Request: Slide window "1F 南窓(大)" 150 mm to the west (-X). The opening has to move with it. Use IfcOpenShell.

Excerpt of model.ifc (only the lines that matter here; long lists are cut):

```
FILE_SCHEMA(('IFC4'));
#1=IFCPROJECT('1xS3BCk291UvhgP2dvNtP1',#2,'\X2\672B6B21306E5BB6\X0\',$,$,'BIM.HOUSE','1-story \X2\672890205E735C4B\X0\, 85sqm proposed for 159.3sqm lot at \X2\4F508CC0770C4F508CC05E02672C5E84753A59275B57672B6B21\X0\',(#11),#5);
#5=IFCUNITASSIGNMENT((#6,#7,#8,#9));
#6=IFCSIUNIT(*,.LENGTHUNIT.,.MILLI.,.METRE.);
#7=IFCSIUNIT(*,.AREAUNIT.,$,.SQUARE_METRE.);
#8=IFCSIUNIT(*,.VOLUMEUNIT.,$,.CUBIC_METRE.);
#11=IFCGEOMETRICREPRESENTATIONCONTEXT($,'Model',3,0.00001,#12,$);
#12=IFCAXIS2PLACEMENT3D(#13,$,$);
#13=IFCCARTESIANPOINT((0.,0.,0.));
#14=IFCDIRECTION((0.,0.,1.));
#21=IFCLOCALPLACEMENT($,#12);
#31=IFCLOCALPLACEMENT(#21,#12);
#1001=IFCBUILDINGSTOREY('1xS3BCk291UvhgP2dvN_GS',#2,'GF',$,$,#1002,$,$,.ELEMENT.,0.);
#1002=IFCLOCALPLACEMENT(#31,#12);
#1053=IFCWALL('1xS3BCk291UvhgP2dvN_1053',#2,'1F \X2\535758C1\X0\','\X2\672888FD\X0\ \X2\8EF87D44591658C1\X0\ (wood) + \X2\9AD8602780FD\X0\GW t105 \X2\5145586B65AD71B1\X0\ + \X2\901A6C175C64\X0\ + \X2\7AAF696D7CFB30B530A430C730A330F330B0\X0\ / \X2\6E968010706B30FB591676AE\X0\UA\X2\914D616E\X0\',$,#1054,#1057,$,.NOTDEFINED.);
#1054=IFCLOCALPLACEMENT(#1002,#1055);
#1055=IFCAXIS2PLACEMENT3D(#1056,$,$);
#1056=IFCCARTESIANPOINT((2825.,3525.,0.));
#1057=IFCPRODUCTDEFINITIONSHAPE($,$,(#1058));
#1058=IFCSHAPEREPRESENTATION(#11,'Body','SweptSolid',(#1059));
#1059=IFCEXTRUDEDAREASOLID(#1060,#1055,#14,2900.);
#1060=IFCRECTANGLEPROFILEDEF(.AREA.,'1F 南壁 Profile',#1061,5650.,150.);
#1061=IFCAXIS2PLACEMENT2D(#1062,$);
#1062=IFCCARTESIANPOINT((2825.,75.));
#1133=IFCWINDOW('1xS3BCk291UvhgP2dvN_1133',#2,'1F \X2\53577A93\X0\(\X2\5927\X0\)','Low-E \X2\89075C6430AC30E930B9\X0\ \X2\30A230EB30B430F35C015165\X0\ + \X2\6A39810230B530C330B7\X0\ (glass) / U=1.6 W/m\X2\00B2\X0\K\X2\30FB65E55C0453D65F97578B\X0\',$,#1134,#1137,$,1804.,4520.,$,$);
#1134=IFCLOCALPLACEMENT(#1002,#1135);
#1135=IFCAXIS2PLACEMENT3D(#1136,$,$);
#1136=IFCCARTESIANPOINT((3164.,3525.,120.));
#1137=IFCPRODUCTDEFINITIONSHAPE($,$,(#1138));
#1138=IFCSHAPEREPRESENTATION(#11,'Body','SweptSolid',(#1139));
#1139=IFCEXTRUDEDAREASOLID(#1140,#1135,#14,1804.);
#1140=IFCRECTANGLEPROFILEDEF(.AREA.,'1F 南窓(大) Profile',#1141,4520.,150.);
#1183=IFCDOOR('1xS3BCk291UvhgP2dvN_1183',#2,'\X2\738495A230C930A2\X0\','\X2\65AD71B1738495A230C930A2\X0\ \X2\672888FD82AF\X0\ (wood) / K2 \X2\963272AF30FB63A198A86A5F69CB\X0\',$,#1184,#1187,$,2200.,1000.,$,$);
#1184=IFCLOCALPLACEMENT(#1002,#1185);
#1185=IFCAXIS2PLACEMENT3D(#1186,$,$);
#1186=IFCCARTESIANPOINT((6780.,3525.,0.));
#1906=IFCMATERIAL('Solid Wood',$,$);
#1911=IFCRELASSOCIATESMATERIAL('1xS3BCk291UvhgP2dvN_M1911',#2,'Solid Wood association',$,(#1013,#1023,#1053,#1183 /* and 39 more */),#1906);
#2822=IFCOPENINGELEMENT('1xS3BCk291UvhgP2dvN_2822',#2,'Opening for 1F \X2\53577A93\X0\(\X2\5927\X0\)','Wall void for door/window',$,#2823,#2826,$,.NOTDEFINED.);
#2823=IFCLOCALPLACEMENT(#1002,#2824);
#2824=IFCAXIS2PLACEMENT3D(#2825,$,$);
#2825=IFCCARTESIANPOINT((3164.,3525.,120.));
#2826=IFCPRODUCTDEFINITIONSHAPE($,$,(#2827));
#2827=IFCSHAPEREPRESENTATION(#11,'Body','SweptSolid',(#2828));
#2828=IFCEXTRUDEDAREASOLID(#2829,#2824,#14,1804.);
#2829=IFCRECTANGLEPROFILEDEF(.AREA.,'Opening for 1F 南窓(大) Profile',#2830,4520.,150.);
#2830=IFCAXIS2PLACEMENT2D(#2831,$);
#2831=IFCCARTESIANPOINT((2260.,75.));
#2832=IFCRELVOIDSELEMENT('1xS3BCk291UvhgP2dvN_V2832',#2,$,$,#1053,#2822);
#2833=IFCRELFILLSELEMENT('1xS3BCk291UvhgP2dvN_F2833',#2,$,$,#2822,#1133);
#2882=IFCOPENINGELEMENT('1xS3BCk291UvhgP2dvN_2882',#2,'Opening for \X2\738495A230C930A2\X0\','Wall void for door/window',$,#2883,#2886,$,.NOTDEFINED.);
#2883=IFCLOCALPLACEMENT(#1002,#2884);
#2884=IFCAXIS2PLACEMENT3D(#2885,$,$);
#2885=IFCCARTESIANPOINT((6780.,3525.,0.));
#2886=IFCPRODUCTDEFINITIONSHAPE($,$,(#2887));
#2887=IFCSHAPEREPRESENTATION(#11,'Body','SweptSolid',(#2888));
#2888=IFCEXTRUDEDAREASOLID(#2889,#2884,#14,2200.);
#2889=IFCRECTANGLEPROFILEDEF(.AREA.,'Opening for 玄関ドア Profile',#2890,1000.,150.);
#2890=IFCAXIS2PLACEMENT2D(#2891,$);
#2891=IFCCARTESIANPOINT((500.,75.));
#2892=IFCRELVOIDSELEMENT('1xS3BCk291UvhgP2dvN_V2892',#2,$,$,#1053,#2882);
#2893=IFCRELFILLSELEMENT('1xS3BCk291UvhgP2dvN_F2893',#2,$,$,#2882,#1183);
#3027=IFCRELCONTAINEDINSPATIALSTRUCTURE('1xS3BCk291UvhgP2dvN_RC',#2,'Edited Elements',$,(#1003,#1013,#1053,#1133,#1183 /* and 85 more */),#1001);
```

```python
import ifcopenshell
import ifcopenshell.api.geometry
import ifcopenshell.util.placement
import ifcopenshell.util.unit

model = ifcopenshell.open("model.ifc")
unit_scale = ifcopenshell.util.unit.calculate_unit_scale(model)

window = model.by_guid("1xS3BCk291UvhgP2dvN_1133")
opening = window.FillsVoids[0].RelatingOpeningElement
wall = opening.VoidsElements[0].RelatingBuildingElement

wall_matrix = ifcopenshell.util.placement.get_local_placement(wall.ObjectPlacement)
shift = wall_matrix[:3, 0] * -0.15 / unit_scale
before = ifcopenshell.util.placement.get_local_placement(window.ObjectPlacement)[:3, 3].copy()

# The window is not placed relative to its opening, so move both.
for product in (opening, window):
    matrix = ifcopenshell.util.placement.get_local_placement(product.ObjectPlacement)
    matrix[:3, 3] += shift
    ifcopenshell.api.geometry.edit_object_placement(model, product=product, matrix=matrix, is_si=False)

after = ifcopenshell.util.placement.get_local_placement(window.ObjectPlacement)[:3, 3]
print("window moved by", (after - before).round(3) + 0.0)

model.write("model_v2.ifc")
```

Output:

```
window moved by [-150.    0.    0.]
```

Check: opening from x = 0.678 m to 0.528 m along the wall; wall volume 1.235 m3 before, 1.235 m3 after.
